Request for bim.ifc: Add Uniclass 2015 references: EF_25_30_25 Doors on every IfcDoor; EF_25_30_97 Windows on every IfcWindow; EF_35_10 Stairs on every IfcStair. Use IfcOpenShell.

First a look at what the model holds.

```python
import ifcopenshell

model = ifcopenshell.open("bim.ifc")
print(model.schema)
print("classifications:", [c.Name for c in model.by_type("IfcClassification")])
for ifc_class in ("IfcDoor", "IfcRoof", "IfcStair", "IfcWall", "IfcWindow"):
    print(ifc_class, len(model.by_type(ifc_class)))
```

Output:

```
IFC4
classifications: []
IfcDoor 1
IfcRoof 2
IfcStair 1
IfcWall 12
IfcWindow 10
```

```python
import ifcopenshell
import ifcopenshell.api.classification

model = ifcopenshell.open("bim.ifc")

system = ifcopenshell.api.classification.add_classification(model, classification="Uniclass 2015")

codes = {
    "IfcDoor": ("EF_25_30_25", "Doors"),
    "IfcWindow": ("EF_25_30_97", "Windows"),
    "IfcStair": ("EF_35_10", "Stairs"),
}
for ifc_class, (code, name) in codes.items():
    products = model.by_type(ifc_class)
    ifcopenshell.api.classification.add_reference(
        model, products=products, classification=system, identification=code, name=name
    )
    print(code, len(products))

model.write("bim_v2.ifc")
```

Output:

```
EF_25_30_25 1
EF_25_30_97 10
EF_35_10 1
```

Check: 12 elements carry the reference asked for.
